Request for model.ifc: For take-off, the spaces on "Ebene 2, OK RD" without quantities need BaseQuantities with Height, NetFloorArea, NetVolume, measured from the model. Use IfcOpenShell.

First a look at what the model holds.

```python
import ifcopenshell
import ifcopenshell.util.element
import ifcopenshell.util.unit

model = ifcopenshell.open("model.ifc")
print(model.schema)
for unit_type in ("LENGTHUNIT", "AREAUNIT", "VOLUMEUNIT"):
    print(unit_type, ifcopenshell.util.unit.calculate_unit_scale(model, unit_type))
storey = next(s for s in model.by_type("IfcBuildingStorey") if s.Name == "Ebene 2, OK RD")
spaces = [e for e in ifcopenshell.util.element.get_decomposition(storey) if e.is_a("IfcSpace")]
for e in sorted(spaces, key=lambda e: e.id()):
    print(e.id(), e.is_a(), e.Name, list(ifcopenshell.util.element.get_psets(e, qtos_only=True)), sep=" | ")
```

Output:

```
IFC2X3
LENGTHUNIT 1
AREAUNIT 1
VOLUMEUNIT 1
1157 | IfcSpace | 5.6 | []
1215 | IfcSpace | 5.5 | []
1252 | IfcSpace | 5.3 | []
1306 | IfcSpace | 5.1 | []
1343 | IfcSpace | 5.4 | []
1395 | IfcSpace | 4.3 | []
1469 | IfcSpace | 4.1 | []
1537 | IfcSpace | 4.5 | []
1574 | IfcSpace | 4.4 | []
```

```python
import ifcopenshell
import ifcopenshell.api.pset
import ifcopenshell.geom
import ifcopenshell.util.element
import ifcopenshell.util.shape
import ifcopenshell.util.unit

model = ifcopenshell.open("model.ifc")
unit_scale = ifcopenshell.util.unit.calculate_unit_scale(model)
area_scale = ifcopenshell.util.unit.calculate_unit_scale(model, "AREAUNIT")
volume_scale = ifcopenshell.util.unit.calculate_unit_scale(model, "VOLUMEUNIT")
settings = ifcopenshell.geom.settings()

storey = next(s for s in model.by_type("IfcBuildingStorey") if s.Name == "Ebene 2, OK RD")
spaces = [e for e in ifcopenshell.util.element.get_decomposition(storey) if e.is_a("IfcSpace")]

for e in sorted(spaces, key=lambda e: e.id()):
    if ifcopenshell.util.element.get_psets(e, qtos_only=True, should_inherit=False):
        continue
    # Geometry comes back in metres, in the element's own axes.
    shape = ifcopenshell.geom.create_shape(settings, e)
    values = {
        "Height": ifcopenshell.util.shape.get_z(shape.geometry) / unit_scale,
        "NetFloorArea": ifcopenshell.util.shape.get_footprint_area(shape.geometry) / area_scale,
        "NetVolume": ifcopenshell.util.shape.get_volume(shape.geometry) / volume_scale,
    }
    qto = ifcopenshell.api.pset.add_qto(model, product=e, name="BaseQuantities")
    ifcopenshell.api.pset.edit_qto(model, qto=qto, properties=values)
    print(e.id(), {k: round(v, 3) for k, v in values.items()})

model.write("model_updated.ifc")
```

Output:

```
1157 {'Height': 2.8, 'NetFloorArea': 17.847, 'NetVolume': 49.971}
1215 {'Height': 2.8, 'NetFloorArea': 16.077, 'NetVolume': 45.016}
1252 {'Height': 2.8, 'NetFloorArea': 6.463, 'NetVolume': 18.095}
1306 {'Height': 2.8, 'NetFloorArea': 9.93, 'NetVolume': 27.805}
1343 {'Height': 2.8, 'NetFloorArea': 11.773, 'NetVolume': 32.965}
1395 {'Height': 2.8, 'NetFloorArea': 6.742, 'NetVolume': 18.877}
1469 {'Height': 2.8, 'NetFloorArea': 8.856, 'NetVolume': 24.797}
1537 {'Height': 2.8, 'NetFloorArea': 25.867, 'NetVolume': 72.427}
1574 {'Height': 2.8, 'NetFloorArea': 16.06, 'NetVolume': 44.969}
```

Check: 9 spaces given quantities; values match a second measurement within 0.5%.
